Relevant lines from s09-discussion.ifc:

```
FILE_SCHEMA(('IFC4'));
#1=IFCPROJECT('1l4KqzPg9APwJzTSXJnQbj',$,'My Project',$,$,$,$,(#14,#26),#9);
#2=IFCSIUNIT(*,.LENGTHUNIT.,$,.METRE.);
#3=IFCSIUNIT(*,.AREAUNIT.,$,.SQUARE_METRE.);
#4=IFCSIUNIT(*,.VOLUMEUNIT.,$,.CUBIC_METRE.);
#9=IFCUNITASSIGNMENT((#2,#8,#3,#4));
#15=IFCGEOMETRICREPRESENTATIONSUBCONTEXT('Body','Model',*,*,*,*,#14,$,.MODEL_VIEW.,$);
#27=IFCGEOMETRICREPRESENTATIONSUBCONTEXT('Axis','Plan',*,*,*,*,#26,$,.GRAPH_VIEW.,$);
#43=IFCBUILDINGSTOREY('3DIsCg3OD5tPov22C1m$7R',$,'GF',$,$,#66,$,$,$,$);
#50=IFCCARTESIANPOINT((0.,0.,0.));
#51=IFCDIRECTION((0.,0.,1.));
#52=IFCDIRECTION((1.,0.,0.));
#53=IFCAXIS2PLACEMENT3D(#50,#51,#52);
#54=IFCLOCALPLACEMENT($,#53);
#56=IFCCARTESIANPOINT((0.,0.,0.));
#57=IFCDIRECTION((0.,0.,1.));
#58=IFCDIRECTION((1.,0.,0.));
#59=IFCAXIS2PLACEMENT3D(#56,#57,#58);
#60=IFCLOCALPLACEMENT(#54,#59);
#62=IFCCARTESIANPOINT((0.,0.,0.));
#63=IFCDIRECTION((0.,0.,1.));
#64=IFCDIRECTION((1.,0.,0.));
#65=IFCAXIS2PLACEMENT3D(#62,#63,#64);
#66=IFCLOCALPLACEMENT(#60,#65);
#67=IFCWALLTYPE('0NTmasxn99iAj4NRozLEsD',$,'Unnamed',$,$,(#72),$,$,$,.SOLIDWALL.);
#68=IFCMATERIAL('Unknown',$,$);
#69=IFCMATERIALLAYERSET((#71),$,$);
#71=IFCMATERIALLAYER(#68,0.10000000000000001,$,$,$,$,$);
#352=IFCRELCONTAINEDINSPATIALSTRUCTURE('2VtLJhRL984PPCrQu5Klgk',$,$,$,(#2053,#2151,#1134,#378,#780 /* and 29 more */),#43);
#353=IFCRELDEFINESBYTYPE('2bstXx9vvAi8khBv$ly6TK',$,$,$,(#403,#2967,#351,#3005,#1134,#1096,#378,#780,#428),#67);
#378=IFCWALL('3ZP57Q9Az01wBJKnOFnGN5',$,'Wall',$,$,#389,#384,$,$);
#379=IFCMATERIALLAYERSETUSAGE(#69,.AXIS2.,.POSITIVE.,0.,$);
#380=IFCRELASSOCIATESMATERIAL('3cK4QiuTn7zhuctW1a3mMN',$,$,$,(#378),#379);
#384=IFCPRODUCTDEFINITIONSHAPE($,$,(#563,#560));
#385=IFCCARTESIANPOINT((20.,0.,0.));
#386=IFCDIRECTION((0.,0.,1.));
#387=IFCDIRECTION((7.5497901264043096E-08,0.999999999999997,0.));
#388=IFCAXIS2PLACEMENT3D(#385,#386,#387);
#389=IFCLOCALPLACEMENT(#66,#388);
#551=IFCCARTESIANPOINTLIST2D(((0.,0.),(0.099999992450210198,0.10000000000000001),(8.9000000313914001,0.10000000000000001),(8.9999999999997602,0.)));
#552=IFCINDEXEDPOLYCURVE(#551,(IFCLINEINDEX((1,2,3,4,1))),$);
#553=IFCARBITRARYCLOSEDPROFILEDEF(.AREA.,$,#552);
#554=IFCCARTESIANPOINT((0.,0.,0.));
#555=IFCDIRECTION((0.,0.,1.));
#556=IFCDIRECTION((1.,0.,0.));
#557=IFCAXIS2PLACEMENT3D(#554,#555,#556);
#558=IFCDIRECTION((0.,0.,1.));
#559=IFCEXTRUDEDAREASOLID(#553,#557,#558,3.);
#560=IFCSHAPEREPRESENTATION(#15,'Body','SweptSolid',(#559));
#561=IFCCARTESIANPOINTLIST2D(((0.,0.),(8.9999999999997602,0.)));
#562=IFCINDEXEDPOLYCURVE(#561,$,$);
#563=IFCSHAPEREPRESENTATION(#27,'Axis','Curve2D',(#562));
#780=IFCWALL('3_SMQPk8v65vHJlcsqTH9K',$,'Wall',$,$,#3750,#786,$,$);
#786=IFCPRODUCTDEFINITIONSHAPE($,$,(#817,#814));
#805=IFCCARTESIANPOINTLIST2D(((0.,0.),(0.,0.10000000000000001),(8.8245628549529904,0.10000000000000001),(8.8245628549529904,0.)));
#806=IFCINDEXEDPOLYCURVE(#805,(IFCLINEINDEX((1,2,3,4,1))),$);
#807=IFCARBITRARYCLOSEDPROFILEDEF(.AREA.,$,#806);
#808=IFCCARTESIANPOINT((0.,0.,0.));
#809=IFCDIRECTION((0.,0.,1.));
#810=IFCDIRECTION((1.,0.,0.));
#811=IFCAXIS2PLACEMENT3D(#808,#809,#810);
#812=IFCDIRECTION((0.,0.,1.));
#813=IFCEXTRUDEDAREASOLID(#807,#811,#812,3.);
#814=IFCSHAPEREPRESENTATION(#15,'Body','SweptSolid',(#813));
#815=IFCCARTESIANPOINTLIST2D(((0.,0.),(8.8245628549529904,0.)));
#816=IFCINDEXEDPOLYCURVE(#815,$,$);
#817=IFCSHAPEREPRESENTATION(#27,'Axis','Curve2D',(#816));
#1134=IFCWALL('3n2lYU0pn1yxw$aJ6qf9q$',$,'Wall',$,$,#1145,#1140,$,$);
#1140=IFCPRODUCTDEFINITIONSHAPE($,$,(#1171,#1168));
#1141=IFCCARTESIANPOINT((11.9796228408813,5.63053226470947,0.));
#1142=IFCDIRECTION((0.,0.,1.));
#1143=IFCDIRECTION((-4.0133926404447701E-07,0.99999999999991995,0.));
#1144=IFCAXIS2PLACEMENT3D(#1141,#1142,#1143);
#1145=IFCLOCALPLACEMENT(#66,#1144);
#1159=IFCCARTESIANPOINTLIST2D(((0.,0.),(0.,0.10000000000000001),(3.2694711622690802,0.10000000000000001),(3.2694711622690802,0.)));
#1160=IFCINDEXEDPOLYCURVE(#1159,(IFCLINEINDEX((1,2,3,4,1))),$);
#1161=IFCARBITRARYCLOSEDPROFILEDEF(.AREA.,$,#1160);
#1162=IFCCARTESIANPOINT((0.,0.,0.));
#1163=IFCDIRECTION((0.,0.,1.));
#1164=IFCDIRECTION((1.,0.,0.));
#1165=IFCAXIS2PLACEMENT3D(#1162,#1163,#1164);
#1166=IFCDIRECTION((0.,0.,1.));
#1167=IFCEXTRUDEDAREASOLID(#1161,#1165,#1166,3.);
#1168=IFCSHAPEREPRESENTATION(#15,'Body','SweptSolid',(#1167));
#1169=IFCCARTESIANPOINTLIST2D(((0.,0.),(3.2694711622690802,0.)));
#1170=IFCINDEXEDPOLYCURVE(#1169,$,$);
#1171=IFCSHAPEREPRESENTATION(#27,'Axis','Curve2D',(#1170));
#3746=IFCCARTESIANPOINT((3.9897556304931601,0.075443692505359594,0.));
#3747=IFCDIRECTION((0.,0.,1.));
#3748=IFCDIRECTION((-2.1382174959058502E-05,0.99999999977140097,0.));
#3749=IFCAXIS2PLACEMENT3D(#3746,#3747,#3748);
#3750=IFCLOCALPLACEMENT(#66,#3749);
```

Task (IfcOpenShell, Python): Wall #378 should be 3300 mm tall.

```python
import ifcopenshell
import ifcopenshell.geom
import ifcopenshell.util.representation
import ifcopenshell.util.shape
import ifcopenshell.util.unit

model = ifcopenshell.open("s09-discussion.ifc")
unit_scale = ifcopenshell.util.unit.calculate_unit_scale(model)
settings = ifcopenshell.geom.settings()


def volume(element):
    """Net volume in cubic metres, openings subtracted."""
    shape = ifcopenshell.geom.create_shape(settings, element)
    return ifcopenshell.util.shape.get_volume(shape.geometry)


wall = model.by_id(378)
before = volume(wall)

body = ifcopenshell.util.representation.get_representation(wall, "Model", "Body")
solid = body.Items[0]
old_height = solid.Depth
solid.Depth = 3.3 / unit_scale
after = volume(wall)

print(f"height {old_height:g} -> {solid.Depth:g}, volume {before:.3f} -> {after:.3f} m3")

model.write("s09-discussion_updated.ifc")
```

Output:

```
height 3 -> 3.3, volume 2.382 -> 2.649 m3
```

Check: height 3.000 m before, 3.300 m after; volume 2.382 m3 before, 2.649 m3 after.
